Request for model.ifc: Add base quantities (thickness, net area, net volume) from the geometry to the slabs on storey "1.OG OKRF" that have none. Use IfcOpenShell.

First a look at what the model holds.

```python
import ifcopenshell
import ifcopenshell.util.element
import ifcopenshell.util.unit

model = ifcopenshell.open("model.ifc")
print(model.schema)
for unit_type in ("LENGTHUNIT", "AREAUNIT", "VOLUMEUNIT"):
    print(unit_type, ifcopenshell.util.unit.calculate_unit_scale(model, unit_type))
storey = next(s for s in model.by_type("IfcBuildingStorey") if s.Name == "1.OG OKRF")
slabs = [e for e in ifcopenshell.util.element.get_decomposition(storey) if e.is_a("IfcSlab")]
for e in sorted(slabs, key=lambda e: e.id()):
    print(e.id(), e.is_a(), e.Name, list(ifcopenshell.util.element.get_psets(e, qtos_only=True)), sep=" | ")
```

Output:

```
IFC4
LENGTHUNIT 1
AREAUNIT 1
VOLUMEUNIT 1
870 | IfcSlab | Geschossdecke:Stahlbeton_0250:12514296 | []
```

```python
import ifcopenshell
import ifcopenshell.api.pset
import ifcopenshell.geom
import ifcopenshell.util.element
import ifcopenshell.util.shape
import ifcopenshell.util.unit

model = ifcopenshell.open("model.ifc")
unit_scale = ifcopenshell.util.unit.calculate_unit_scale(model)
area_scale = ifcopenshell.util.unit.calculate_unit_scale(model, "AREAUNIT")
volume_scale = ifcopenshell.util.unit.calculate_unit_scale(model, "VOLUMEUNIT")
settings = ifcopenshell.geom.settings()

storey = next(s for s in model.by_type("IfcBuildingStorey") if s.Name == "1.OG OKRF")
slabs = [e for e in ifcopenshell.util.element.get_decomposition(storey) if e.is_a("IfcSlab")]

for e in sorted(slabs, key=lambda e: e.id()):
    if ifcopenshell.util.element.get_psets(e, qtos_only=True, should_inherit=False):
        continue
    # Geometry comes back in metres, in the element's own axes.
    shape = ifcopenshell.geom.create_shape(settings, e)
    values = {
        "Width": ifcopenshell.util.shape.get_z(shape.geometry) / unit_scale,
        "NetArea": ifcopenshell.util.shape.get_footprint_area(shape.geometry) / area_scale,
        "NetVolume": ifcopenshell.util.shape.get_volume(shape.geometry) / volume_scale,
    }
    qto = ifcopenshell.api.pset.add_qto(model, product=e, name="Qto_SlabBaseQuantities")
    ifcopenshell.api.pset.edit_qto(model, qto=qto, properties=values)
    print(e.id(), {k: round(v, 3) for k, v in values.items()})

model.write("model_updated.ifc")
```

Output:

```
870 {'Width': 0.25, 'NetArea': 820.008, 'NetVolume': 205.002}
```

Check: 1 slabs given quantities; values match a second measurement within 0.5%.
